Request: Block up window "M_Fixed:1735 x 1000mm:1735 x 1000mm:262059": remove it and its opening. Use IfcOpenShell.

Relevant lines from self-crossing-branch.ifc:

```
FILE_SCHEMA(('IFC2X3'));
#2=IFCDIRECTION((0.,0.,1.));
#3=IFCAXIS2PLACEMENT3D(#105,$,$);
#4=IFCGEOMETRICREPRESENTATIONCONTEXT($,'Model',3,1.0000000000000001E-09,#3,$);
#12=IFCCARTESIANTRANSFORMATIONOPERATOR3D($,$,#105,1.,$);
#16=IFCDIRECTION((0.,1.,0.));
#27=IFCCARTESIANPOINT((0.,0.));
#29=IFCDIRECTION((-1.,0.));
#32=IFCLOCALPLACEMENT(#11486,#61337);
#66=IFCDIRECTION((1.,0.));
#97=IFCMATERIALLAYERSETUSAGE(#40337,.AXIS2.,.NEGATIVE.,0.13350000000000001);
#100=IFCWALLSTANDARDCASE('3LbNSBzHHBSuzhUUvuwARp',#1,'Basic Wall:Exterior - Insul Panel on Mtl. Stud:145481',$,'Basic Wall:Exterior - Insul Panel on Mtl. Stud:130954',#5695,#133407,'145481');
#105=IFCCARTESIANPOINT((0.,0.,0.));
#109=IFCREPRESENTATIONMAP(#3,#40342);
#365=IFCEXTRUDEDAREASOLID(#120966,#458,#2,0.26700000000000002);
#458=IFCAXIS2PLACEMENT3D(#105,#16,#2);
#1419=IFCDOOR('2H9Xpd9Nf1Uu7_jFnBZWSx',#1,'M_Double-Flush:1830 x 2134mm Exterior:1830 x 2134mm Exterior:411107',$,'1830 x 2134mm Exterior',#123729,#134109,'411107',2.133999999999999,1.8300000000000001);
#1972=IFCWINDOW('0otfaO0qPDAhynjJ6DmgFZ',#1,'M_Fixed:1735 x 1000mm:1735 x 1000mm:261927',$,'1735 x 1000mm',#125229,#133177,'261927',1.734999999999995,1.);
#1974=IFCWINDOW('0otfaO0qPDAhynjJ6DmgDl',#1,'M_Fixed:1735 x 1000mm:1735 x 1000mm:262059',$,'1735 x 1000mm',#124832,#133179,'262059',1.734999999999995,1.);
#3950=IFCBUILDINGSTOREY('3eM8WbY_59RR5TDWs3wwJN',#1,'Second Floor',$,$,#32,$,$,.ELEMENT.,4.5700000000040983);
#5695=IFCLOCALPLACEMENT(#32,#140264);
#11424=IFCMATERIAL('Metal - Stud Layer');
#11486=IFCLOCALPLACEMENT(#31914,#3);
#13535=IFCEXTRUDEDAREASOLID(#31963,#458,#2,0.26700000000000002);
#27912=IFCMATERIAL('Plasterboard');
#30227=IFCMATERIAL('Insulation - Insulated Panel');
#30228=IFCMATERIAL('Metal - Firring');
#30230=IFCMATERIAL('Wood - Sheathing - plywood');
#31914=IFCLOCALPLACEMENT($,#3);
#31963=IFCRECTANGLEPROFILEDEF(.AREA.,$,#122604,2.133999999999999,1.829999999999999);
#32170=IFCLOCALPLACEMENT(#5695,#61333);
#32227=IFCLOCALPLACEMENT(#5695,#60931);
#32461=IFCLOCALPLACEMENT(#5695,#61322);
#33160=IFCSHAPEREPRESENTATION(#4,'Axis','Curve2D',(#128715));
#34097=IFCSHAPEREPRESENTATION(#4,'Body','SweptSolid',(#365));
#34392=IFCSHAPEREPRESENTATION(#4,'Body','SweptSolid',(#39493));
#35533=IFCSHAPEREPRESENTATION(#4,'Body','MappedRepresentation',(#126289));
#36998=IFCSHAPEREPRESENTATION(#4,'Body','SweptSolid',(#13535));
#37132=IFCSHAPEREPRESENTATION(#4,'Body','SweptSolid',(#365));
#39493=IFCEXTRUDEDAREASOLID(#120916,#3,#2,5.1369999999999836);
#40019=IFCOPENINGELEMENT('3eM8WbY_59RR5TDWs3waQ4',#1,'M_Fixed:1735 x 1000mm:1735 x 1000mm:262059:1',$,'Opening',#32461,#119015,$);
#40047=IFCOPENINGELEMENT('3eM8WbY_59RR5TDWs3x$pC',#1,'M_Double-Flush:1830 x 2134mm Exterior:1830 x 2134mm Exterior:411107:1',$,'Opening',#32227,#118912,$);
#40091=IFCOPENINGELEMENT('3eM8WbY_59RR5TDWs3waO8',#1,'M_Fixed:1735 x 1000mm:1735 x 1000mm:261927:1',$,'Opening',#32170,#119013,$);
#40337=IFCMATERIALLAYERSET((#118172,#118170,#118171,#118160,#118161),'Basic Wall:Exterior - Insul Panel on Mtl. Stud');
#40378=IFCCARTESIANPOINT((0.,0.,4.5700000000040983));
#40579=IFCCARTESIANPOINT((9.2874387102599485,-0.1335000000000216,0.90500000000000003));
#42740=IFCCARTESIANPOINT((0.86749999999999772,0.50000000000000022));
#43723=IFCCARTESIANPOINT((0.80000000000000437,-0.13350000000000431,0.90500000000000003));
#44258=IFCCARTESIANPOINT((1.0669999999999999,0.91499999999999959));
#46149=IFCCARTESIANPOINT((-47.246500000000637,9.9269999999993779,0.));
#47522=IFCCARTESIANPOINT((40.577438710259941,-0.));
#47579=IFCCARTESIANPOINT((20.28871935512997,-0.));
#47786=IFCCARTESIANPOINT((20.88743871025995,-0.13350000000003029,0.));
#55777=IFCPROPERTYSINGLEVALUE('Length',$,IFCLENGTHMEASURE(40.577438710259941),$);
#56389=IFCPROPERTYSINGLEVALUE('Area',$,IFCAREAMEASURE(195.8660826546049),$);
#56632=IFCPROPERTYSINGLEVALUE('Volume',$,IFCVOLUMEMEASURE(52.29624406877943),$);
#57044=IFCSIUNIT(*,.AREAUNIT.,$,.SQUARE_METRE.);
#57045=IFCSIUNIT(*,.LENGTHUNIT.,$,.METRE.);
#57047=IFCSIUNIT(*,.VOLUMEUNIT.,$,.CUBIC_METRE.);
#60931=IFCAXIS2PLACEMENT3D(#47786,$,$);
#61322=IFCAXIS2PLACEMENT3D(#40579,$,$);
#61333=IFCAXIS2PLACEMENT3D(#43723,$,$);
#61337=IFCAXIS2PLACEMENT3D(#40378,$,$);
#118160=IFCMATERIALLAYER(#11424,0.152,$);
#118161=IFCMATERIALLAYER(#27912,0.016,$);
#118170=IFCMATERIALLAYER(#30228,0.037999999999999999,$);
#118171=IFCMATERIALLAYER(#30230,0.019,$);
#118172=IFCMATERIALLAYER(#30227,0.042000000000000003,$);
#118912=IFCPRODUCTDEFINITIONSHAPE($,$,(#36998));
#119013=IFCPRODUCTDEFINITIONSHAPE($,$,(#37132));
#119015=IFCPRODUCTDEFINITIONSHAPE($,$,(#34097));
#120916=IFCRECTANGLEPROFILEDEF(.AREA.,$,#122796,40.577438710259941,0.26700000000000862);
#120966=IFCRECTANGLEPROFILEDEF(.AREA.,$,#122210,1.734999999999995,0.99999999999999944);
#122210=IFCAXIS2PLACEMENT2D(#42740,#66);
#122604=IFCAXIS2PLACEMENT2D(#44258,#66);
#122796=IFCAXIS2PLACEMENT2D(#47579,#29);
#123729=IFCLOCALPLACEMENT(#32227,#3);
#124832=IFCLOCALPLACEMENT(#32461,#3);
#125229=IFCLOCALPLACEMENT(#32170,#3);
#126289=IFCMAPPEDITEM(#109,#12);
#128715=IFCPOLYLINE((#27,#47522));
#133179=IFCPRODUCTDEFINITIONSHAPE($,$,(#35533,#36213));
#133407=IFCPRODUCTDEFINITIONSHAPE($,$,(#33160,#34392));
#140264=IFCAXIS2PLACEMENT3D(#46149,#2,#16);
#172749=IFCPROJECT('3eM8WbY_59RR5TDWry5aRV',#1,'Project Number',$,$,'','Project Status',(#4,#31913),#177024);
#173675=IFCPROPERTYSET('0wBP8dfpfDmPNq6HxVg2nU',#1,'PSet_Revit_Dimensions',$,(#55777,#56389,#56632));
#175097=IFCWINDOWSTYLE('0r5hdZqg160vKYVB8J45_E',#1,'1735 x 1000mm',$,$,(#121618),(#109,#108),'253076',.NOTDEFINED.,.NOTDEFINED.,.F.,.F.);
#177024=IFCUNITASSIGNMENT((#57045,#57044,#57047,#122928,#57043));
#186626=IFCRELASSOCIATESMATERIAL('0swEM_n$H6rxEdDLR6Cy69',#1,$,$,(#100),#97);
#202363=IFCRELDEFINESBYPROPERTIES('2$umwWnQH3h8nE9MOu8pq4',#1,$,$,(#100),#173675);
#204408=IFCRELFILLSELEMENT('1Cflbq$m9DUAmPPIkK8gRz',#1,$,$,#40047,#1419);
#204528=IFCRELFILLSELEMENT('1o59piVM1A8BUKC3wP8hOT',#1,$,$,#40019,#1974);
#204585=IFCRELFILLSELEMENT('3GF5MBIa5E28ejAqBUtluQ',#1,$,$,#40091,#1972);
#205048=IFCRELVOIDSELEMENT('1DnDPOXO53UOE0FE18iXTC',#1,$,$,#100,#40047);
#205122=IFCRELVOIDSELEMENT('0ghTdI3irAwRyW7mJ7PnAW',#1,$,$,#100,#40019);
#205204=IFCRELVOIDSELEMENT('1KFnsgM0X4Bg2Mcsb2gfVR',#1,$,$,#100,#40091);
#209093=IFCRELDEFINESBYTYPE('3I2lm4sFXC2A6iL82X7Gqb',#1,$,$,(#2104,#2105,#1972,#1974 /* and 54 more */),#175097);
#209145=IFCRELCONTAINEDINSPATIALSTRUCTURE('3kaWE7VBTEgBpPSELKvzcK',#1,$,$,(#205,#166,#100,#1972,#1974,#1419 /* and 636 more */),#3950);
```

```python
import ifcopenshell
import ifcopenshell.api.feature
import ifcopenshell.api.pset
import ifcopenshell.api.root
import ifcopenshell.geom
import ifcopenshell.util.element
import ifcopenshell.util.shape
import ifcopenshell.util.unit

model = ifcopenshell.open("self-crossing-branch.ifc")
area_scale = ifcopenshell.util.unit.calculate_unit_scale(model, "AREAUNIT")
volume_scale = ifcopenshell.util.unit.calculate_unit_scale(model, "VOLUMEUNIT")
settings = ifcopenshell.geom.settings()


def volume(element):
    """Net volume in cubic metres, openings subtracted."""
    shape = ifcopenshell.geom.create_shape(settings, element)
    return ifcopenshell.util.shape.get_volume(shape.geometry)


window = model.by_guid("0otfaO0qPDAhynjJ6DmgDl")
opening = window.FillsVoids[0].RelatingOpeningElement
wall = opening.VoidsElements[0].RelatingBuildingElement
before = volume(wall)

ifcopenshell.api.root.remove_product(model, product=window)
ifcopenshell.api.feature.remove_feature(model, feature=opening)

after = volume(wall)
thickness = 0.267  # wall thickness in metres

# Update the wall's stored quantities.
pset = model.by_id(ifcopenshell.util.element.get_pset(wall, "PSet_Revit_Dimensions", should_inherit=False)["id"])
ifcopenshell.api.pset.edit_pset(model, pset=pset, properties={
    "Area": model.create_entity("IfcAreaMeasure", after / thickness / area_scale),
    "Volume": model.create_entity("IfcVolumeMeasure", after / volume_scale),
})

print(f"wall volume {before:.3f} -> {after:.3f} m3")

model.write("self-crossing-branch_updated.ifc")
```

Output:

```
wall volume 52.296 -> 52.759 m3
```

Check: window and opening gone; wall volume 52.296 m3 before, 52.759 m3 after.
